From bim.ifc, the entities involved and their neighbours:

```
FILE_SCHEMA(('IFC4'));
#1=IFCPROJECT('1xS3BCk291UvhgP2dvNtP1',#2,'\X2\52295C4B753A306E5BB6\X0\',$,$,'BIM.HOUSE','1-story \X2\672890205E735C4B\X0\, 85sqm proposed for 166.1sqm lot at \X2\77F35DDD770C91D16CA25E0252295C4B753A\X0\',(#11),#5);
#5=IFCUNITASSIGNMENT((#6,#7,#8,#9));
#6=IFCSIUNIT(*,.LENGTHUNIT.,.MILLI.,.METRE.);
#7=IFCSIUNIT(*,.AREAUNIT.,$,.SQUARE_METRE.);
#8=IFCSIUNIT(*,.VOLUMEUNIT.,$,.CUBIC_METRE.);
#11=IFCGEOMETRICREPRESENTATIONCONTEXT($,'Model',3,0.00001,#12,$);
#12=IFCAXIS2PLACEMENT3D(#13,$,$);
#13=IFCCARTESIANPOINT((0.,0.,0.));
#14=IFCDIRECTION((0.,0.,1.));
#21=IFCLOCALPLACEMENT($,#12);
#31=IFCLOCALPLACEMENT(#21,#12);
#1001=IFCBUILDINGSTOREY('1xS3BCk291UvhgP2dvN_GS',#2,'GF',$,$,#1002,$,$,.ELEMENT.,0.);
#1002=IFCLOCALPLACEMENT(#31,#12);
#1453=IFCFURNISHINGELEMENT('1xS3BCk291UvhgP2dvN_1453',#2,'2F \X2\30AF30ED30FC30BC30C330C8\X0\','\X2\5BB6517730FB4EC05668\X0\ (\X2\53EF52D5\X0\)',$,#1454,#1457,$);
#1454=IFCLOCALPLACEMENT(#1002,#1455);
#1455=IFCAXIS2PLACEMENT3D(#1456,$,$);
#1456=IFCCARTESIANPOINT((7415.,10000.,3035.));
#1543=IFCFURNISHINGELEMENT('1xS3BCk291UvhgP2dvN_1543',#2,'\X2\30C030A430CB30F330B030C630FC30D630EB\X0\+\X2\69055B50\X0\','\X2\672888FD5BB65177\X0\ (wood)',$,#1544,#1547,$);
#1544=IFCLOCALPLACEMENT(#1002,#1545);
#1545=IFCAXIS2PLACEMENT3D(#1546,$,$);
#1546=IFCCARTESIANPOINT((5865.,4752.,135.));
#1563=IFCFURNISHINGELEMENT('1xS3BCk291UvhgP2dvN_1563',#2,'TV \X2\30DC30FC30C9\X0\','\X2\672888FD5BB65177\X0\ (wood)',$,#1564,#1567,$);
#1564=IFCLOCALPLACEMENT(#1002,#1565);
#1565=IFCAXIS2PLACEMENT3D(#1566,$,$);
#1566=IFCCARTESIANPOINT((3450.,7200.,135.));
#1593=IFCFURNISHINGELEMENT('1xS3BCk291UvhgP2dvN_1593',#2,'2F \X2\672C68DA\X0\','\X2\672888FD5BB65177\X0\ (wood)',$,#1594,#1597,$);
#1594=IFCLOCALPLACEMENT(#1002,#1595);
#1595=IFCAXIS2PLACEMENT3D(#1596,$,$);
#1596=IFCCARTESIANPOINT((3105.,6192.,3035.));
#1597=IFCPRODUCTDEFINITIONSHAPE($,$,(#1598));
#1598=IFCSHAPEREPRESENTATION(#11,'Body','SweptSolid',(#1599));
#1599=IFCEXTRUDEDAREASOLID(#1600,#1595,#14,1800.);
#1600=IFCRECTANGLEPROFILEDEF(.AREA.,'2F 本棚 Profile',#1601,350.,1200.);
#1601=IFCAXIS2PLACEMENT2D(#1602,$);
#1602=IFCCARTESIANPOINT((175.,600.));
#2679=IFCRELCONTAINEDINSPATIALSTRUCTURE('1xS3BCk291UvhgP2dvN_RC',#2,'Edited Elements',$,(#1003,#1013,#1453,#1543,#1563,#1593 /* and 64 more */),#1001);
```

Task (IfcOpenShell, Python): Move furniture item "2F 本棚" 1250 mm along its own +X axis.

```python
import ifcopenshell
import ifcopenshell.api.geometry
import ifcopenshell.util.placement
import ifcopenshell.util.unit

model = ifcopenshell.open("bim.ifc")
unit_scale = ifcopenshell.util.unit.calculate_unit_scale(model)

item = model.by_guid("1xS3BCk291UvhgP2dvN_1593")
matrix = ifcopenshell.util.placement.get_local_placement(item.ObjectPlacement)
matrix[:3, 3] += matrix[:3, 0] * 1.25 / unit_scale
ifcopenshell.api.geometry.edit_object_placement(model, product=item, matrix=matrix, is_si=False)

print(ifcopenshell.util.placement.get_local_placement(item.ObjectPlacement).round(3) + 0.0)

model.write("bim_updated.ifc")
```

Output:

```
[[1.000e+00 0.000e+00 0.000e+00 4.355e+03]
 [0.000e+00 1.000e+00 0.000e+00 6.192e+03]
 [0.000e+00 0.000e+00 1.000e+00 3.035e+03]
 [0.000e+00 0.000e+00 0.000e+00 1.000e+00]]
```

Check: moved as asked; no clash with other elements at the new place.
